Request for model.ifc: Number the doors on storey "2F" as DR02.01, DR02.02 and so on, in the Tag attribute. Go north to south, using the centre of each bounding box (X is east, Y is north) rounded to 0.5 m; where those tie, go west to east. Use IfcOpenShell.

First a look at what the model holds.

```python
import ifcopenshell
import ifcopenshell.util.element
import ifcopenshell.util.placement

model = ifcopenshell.open("model.ifc")
print(model.schema)
storey = next(s for s in model.by_type("IfcBuildingStorey") if s.Name == "2F")
doors = [e for e in ifcopenshell.util.element.get_decomposition(storey) if e.is_a("IfcDoor")]
for e in sorted(doors, key=lambda e: e.id()):
    origin = ifcopenshell.util.placement.get_local_placement(e.ObjectPlacement)[:3, 3]
    print(e.id(), e.Tag, e.Name, origin.round(2) + 0.0, sep=" | ")
```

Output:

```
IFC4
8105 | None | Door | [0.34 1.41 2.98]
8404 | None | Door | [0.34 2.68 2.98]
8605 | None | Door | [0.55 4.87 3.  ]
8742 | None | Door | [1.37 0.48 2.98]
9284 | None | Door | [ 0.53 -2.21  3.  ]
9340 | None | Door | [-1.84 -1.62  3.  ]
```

```python
import ifcopenshell
import ifcopenshell.geom
import ifcopenshell.util.element
import ifcopenshell.util.shape

model = ifcopenshell.open("model.ifc")
settings = ifcopenshell.geom.settings()
settings.set("use-world-coords", True)


def centre(element):
    shape = ifcopenshell.geom.create_shape(settings, element)
    return ifcopenshell.util.shape.get_bbox_centroid(shape.geometry)


storey = next(s for s in model.by_type("IfcBuildingStorey") if s.Name == "2F")
doors = [e for e in ifcopenshell.util.element.get_decomposition(storey) if e.is_a("IfcDoor")]

# Insertion points can sit at a corner or the storey origin, so sort by the geometry (in metres).
centres = {e: centre(e) for e in doors}
doors.sort(key=lambda e: (-round(centres[e][1] / 0.5), centres[e][0]))

for i, e in enumerate(doors, start=1):
    number = f"DR02.{i:02d}"
    e.Tag = number
    print(e.id(), number)

model.write("model_rev.ifc")
```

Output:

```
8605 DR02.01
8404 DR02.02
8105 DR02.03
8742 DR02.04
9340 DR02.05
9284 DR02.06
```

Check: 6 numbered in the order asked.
